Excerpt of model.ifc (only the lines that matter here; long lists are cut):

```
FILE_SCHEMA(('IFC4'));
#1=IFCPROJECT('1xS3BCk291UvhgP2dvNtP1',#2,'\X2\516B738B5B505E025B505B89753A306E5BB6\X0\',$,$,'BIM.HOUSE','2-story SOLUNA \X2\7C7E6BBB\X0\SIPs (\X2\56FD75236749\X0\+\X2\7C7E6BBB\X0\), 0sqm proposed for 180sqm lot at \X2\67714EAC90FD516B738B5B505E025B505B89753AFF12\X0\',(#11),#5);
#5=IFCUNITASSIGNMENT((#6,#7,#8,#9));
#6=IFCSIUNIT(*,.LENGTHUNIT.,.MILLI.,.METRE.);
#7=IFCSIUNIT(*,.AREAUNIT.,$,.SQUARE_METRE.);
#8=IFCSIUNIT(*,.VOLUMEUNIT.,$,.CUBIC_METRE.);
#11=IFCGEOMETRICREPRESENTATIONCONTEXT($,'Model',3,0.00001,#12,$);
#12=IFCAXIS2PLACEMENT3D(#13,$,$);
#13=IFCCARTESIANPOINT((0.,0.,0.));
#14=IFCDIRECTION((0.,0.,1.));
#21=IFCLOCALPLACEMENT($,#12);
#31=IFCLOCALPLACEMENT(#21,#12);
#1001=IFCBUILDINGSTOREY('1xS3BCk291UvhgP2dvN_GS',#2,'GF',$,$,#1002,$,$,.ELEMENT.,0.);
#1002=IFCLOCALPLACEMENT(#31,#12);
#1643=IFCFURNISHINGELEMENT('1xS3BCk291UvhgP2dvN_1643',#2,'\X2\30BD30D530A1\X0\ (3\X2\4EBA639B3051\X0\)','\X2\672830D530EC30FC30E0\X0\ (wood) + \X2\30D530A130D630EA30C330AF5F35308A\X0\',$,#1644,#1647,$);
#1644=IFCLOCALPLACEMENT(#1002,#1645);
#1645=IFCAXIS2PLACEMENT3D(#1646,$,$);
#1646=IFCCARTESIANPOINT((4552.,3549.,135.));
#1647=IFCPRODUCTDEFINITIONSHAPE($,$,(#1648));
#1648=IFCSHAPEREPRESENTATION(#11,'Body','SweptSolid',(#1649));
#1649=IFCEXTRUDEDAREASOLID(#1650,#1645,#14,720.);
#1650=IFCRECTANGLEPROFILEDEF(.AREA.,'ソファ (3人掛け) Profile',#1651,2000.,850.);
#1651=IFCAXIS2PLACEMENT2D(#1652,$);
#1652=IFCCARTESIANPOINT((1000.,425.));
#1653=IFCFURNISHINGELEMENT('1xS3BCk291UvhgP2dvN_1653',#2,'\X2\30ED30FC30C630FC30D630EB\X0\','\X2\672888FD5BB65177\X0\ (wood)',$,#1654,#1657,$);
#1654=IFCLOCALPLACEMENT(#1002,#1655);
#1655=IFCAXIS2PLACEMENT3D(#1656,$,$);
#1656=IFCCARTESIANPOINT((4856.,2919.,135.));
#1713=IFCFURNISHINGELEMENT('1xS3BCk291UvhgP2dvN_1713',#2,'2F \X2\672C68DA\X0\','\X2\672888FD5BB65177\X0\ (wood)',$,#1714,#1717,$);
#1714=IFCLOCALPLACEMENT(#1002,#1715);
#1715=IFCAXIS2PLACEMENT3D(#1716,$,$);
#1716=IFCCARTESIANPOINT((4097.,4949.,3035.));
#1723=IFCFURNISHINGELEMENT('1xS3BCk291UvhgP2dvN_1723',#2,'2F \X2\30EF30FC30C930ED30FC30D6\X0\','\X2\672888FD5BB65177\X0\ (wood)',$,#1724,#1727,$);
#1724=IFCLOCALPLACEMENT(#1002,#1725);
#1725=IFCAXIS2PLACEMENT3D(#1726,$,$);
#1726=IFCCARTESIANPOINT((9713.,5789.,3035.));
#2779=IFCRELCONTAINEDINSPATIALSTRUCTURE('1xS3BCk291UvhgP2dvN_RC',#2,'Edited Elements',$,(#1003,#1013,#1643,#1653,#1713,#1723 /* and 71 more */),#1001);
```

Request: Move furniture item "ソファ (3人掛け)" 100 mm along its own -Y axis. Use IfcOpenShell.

```python
import ifcopenshell
import ifcopenshell.api.geometry
import ifcopenshell.util.placement
import ifcopenshell.util.unit

model = ifcopenshell.open("model.ifc")
unit_scale = ifcopenshell.util.unit.calculate_unit_scale(model)

item = model.by_guid("1xS3BCk291UvhgP2dvN_1643")
matrix = ifcopenshell.util.placement.get_local_placement(item.ObjectPlacement)
matrix[:3, 3] -= matrix[:3, 1] * 0.1 / unit_scale
ifcopenshell.api.geometry.edit_object_placement(model, product=item, matrix=matrix, is_si=False)

print(ifcopenshell.util.placement.get_local_placement(item.ObjectPlacement).round(3) + 0.0)

model.write("model_edited.ifc")
```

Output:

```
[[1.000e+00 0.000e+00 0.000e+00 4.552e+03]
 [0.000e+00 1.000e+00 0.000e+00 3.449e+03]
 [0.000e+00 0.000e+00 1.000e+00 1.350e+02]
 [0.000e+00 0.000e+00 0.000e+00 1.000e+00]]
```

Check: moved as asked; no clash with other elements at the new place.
